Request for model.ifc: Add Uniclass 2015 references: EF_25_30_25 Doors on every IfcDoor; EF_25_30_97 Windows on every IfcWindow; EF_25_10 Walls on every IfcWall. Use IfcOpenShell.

First a look at what the model holds.

```python
import ifcopenshell

model = ifcopenshell.open("model.ifc")
print(model.schema)
print("classifications:", [c.Name for c in model.by_type("IfcClassification")])
for ifc_class in ("IfcDoor", "IfcRoof", "IfcStair", "IfcWall", "IfcWindow"):
    print(ifc_class, len(model.by_type(ifc_class)))
```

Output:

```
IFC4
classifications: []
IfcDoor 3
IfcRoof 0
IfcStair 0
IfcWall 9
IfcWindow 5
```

```python
import ifcopenshell
import ifcopenshell.api.classification

model = ifcopenshell.open("model.ifc")

system = ifcopenshell.api.classification.add_classification(model, classification="Uniclass 2015")

codes = {
    "IfcDoor": ("EF_25_30_25", "Doors"),
    "IfcWindow": ("EF_25_30_97", "Windows"),
    "IfcWall": ("EF_25_10", "Walls"),
}
for ifc_class, (code, name) in codes.items():
    products = model.by_type(ifc_class)
    ifcopenshell.api.classification.add_reference(
        model, products=products, classification=system, identification=code, name=name
    )
    print(code, len(products))

model.write("model_rev.ifc")
```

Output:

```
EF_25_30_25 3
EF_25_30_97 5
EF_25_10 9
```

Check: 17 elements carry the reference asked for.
